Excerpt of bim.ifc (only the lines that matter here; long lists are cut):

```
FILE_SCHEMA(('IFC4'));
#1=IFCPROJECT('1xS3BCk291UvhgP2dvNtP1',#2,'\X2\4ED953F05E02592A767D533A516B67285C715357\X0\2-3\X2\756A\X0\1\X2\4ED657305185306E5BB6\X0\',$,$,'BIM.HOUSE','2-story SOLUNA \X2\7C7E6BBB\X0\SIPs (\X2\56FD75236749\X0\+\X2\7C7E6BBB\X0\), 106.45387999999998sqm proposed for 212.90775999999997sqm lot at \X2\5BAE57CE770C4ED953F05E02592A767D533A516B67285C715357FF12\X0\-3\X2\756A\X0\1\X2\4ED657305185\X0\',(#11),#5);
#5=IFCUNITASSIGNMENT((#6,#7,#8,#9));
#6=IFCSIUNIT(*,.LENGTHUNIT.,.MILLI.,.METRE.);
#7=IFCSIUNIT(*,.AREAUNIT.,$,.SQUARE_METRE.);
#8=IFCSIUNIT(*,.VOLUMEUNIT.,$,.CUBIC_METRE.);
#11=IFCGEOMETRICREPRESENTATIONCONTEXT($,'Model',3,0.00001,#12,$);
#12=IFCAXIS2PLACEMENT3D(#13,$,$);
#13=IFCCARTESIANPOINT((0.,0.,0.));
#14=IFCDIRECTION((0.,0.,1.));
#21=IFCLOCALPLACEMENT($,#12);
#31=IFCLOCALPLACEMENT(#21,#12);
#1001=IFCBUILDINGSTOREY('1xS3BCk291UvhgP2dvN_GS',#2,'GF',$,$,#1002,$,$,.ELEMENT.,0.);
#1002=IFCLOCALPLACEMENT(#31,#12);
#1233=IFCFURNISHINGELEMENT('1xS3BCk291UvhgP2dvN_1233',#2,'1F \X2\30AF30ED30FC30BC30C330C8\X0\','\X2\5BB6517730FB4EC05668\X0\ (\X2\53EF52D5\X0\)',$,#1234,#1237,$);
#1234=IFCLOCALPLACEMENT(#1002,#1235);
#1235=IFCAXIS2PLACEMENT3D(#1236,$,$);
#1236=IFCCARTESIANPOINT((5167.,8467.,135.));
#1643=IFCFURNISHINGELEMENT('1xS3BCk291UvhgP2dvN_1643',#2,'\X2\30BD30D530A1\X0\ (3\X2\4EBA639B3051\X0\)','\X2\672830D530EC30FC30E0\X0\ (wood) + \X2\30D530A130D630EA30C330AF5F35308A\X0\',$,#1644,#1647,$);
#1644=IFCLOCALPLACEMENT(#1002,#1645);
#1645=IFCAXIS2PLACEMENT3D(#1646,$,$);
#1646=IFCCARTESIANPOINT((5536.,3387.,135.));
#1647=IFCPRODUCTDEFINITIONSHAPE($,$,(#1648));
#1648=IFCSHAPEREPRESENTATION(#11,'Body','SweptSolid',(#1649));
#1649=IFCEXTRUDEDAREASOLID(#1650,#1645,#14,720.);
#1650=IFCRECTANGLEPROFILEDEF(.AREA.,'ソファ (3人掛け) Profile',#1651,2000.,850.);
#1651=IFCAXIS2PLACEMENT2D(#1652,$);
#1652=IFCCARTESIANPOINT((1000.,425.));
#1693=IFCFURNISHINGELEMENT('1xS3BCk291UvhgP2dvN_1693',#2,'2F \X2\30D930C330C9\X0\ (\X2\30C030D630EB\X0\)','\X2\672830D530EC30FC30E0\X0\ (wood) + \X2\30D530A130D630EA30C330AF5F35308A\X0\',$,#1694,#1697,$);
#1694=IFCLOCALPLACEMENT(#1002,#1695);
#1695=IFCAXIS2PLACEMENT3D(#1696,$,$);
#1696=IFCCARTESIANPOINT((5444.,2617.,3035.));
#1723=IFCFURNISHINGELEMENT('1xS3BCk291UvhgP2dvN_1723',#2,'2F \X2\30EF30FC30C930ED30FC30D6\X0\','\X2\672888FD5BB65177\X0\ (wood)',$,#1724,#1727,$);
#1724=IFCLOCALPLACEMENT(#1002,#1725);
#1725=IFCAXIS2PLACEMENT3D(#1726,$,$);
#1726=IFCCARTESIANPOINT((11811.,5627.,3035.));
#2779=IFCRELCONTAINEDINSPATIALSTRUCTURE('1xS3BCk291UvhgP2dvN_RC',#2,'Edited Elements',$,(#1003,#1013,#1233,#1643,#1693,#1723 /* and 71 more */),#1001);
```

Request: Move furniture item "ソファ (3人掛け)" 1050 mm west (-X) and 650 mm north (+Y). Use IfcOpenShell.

```python
import ifcopenshell
import ifcopenshell.api.geometry
import ifcopenshell.util.placement
import ifcopenshell.util.unit

model = ifcopenshell.open("bim.ifc")
unit_scale = ifcopenshell.util.unit.calculate_unit_scale(model)

item = model.by_id(1643)
matrix = ifcopenshell.util.placement.get_local_placement(item.ObjectPlacement)
matrix[0, 3] -= 1.05 / unit_scale
matrix[1, 3] += 0.65 / unit_scale
ifcopenshell.api.geometry.edit_object_placement(model, product=item, matrix=matrix, is_si=False)

print(ifcopenshell.util.placement.get_local_placement(item.ObjectPlacement).round(3) + 0.0)

model.write("bim-out.ifc")
```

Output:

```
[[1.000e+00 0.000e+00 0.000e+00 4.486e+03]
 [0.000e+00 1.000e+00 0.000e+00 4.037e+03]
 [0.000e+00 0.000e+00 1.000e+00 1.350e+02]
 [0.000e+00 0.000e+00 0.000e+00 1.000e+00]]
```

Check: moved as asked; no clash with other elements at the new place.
